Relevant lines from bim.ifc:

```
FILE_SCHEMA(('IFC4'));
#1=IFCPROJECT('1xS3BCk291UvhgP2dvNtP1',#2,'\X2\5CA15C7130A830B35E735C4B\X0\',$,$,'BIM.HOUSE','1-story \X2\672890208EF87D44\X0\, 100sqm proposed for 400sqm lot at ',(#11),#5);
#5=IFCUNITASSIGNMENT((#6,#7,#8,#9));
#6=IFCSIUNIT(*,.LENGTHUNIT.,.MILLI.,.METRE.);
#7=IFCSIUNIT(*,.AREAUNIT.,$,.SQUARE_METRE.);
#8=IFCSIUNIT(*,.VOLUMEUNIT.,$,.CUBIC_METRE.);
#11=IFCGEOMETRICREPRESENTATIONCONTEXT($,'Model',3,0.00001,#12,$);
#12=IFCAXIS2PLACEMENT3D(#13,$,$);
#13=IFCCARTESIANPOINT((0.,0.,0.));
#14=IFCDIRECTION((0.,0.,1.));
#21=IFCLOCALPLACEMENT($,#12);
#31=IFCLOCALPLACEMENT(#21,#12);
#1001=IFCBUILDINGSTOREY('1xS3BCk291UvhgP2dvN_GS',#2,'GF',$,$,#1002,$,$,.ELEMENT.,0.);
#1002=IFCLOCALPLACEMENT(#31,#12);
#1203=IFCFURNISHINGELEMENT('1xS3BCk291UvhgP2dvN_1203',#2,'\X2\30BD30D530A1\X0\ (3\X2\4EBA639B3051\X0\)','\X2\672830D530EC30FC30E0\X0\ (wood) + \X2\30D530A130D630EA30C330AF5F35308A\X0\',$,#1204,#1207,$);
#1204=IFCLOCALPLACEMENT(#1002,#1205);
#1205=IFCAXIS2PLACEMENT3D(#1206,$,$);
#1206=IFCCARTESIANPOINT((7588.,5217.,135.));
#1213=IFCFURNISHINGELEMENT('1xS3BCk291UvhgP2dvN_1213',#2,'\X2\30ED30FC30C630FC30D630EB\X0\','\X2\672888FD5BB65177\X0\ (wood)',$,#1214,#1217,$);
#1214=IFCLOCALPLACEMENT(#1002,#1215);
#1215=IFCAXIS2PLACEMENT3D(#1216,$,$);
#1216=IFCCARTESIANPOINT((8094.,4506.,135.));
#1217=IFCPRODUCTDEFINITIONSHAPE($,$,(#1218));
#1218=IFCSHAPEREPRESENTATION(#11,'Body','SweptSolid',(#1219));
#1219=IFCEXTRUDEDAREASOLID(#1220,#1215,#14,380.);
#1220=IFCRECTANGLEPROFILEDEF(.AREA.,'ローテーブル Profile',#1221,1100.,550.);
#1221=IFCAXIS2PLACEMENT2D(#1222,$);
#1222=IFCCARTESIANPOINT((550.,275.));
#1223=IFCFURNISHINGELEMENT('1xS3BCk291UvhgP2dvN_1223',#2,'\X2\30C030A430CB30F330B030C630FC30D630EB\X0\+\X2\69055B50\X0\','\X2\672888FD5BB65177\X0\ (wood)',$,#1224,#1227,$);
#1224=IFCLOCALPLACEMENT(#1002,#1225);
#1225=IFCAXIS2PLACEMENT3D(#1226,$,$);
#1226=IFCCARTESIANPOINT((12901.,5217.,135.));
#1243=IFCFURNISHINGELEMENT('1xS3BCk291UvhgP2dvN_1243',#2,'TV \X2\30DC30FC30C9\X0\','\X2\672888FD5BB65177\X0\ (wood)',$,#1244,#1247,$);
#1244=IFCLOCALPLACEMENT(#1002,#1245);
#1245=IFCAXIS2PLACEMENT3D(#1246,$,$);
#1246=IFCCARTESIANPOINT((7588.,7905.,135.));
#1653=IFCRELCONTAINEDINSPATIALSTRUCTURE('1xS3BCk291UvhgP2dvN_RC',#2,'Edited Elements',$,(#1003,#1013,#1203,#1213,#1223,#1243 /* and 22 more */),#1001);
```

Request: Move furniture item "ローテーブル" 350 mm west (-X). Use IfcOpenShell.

```python
import ifcopenshell
import ifcopenshell.api.geometry
import ifcopenshell.util.placement

model = ifcopenshell.open("bim.ifc")

item = model.by_id(1213)
matrix = ifcopenshell.util.placement.get_local_placement(item.ObjectPlacement)
matrix[0, 3] -= 350.0
ifcopenshell.api.geometry.edit_object_placement(model, product=item, matrix=matrix, is_si=False)

print(ifcopenshell.util.placement.get_local_placement(item.ObjectPlacement).round(3) + 0.0)

model.write("bim_updated.ifc")
```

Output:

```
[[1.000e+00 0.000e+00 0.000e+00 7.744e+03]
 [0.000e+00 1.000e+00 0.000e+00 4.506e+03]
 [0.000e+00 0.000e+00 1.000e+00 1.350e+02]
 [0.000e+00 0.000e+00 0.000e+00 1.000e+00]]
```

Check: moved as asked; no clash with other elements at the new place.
